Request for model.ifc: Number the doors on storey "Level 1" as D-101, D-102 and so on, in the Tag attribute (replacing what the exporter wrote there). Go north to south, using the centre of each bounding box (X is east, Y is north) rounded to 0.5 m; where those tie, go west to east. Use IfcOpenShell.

First a look at what the model holds.

```python
import ifcopenshell
import ifcopenshell.util.element
import ifcopenshell.util.placement

model = ifcopenshell.open("model.ifc")
print(model.schema)
storey = next(s for s in model.by_type("IfcBuildingStorey") if s.Name == "Level 1")
doors = [e for e in ifcopenshell.util.element.get_decomposition(storey) if e.is_a("IfcDoor")]
for e in sorted(doors, key=lambda e: e.id()):
    origin = ifcopenshell.util.placement.get_local_placement(e.ObjectPlacement)[:3, 3]
    print(e.id(), e.Tag, e.Name, origin.round(2) + 0.0, sep=" | ")
```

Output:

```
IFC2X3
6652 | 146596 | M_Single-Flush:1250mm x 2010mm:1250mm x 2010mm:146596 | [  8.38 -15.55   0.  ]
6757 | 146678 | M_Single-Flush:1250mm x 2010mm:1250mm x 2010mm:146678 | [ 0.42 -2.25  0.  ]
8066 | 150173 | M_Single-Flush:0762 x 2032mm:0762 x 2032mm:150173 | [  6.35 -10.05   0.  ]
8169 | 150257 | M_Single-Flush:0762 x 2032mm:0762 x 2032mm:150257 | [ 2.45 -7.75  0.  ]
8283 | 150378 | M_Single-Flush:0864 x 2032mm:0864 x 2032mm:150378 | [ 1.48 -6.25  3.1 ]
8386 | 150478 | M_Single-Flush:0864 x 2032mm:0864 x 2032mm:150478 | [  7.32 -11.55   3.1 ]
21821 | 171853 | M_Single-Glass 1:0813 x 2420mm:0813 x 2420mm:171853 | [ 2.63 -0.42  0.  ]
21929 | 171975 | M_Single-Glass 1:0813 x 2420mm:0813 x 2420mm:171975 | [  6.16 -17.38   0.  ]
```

```python
import ifcopenshell
import ifcopenshell.geom
import ifcopenshell.util.element
import ifcopenshell.util.shape

model = ifcopenshell.open("model.ifc")
settings = ifcopenshell.geom.settings()
settings.set("use-world-coords", True)


def centre(element):
    shape = ifcopenshell.geom.create_shape(settings, element)
    return ifcopenshell.util.shape.get_bbox_centroid(shape.geometry)


storey = next(s for s in model.by_type("IfcBuildingStorey") if s.Name == "Level 1")
doors = [e for e in ifcopenshell.util.element.get_decomposition(storey) if e.is_a("IfcDoor")]

# Insertion points can sit at a corner or the storey origin, so sort by the geometry (in metres).
centres = {e: centre(e) for e in doors}
doors.sort(key=lambda e: (-round(centres[e][1] / 0.5), centres[e][0]))

for i, e in enumerate(doors, start=1):
    number = f"D-1{i:02d}"
    e.Tag = number
    print(e.id(), number)

model.write("model_updated.ifc")
```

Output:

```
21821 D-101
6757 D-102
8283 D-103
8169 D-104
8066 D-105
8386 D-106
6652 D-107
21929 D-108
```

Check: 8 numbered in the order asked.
